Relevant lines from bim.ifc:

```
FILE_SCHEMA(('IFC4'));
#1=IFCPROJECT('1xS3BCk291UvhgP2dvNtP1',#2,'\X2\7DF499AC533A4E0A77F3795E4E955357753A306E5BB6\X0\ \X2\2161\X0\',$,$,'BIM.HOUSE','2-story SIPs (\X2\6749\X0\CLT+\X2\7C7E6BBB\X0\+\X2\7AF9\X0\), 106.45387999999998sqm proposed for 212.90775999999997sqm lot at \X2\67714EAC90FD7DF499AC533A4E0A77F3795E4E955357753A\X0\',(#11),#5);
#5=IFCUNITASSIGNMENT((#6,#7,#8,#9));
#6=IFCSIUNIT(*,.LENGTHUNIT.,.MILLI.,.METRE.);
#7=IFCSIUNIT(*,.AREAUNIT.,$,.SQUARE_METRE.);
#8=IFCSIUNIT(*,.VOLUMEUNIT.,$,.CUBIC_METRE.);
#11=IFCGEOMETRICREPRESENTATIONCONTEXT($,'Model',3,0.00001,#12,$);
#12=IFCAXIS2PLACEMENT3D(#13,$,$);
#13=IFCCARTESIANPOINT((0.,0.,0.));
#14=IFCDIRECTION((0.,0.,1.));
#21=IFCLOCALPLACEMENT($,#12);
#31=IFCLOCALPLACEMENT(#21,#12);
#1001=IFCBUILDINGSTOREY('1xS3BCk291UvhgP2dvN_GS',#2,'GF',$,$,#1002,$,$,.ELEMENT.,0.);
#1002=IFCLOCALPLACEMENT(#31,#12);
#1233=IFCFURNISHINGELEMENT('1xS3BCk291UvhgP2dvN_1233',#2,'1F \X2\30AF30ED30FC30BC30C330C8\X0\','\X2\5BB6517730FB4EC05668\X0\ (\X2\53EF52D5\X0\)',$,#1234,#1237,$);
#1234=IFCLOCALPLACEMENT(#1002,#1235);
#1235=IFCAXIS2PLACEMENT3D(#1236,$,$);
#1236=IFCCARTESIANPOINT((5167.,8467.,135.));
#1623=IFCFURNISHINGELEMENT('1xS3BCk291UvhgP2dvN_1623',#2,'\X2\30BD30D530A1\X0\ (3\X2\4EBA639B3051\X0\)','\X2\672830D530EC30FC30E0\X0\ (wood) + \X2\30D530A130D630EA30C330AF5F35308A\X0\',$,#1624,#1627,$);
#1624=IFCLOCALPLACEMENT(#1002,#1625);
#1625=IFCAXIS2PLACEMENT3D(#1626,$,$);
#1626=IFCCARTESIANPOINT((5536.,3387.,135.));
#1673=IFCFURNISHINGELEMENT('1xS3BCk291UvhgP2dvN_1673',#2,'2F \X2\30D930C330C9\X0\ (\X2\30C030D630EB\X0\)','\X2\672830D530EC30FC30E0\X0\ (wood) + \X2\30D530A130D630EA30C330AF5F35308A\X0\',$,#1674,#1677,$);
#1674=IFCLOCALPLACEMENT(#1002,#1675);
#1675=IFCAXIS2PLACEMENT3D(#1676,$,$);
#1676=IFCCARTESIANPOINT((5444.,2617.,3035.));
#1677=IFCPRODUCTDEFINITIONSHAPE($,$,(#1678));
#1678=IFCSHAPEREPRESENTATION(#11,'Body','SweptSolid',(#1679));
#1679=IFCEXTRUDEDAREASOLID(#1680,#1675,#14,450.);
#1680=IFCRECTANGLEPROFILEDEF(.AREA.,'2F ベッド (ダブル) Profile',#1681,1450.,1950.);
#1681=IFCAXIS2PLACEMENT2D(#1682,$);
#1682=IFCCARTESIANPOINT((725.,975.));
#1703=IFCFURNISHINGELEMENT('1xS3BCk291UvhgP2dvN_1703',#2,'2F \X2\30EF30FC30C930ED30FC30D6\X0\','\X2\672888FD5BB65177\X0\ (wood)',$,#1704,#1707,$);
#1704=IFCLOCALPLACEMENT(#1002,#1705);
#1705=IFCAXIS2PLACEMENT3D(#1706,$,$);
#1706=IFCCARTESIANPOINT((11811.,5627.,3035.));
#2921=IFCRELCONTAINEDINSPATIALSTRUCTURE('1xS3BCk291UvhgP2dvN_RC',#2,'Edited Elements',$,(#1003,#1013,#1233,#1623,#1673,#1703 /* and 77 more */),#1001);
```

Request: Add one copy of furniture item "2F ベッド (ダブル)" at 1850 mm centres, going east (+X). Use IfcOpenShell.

```python
import numpy as np
import ifcopenshell
import ifcopenshell.api.geometry
import ifcopenshell.api.root
import ifcopenshell.util.element
import ifcopenshell.util.placement
import ifcopenshell.util.unit

model = ifcopenshell.open("bim.ifc")
unit_scale = ifcopenshell.util.unit.calculate_unit_scale(model)


def reuse_history(source, copy):
    """copy_class also copies each property set's owner history, people and application; keep the originals."""
    for rel in copy.IsDefinedBy:
        if rel.is_a("IfcRelDefinesByProperties") and (history := rel.RelatingPropertyDefinition.OwnerHistory):
            rel.RelatingPropertyDefinition.OwnerHistory = source.OwnerHistory
            ifcopenshell.util.element.remove_deep2(model, history)


source = model.by_guid("1xS3BCk291UvhgP2dvN_1673")
base = ifcopenshell.util.placement.get_local_placement(source.ObjectPlacement)
step = np.array([1.0, 0.0, 0.0]) * 1.85 / unit_scale

for i in range(1, 2):
    copy = ifcopenshell.api.root.copy_class(model, product=source)
    copy.Representation = ifcopenshell.util.element.copy_deep(
        model, source.Representation, exclude=["IfcGeometricRepresentationContext", "IfcRepresentationMap"]
    )
    reuse_history(source, copy)
    matrix = base.copy()
    matrix[:3, 3] += i * step
    print("added at", matrix[:3, 3].round(3) + 0.0)
    ifcopenshell.api.geometry.edit_object_placement(model, product=copy, matrix=matrix, is_si=False)

model.write("bim_edited.ifc")
```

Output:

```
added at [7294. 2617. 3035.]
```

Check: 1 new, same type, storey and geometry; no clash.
